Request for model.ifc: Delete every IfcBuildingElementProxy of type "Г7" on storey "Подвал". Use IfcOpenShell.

First a look at what the model holds.

```python
import ifcopenshell
import ifcopenshell.util.element

model = ifcopenshell.open("model.ifc")
print(model.schema)
storey = next(s for s in model.by_type("IfcBuildingStorey") if s.Name == "Подвал")
proxies = [e for e in ifcopenshell.util.element.get_decomposition(storey) if e.is_a("IfcBuildingElementProxy")]
seen = {}
for e in proxies:
    element_type = ifcopenshell.util.element.get_type(e)
    name = element_type.Name if element_type not in (None, e) else None
    seen[name] = seen.get(name, 0) + 1
for name, count in sorted(seen.items(), key=str):
    print(count, "x", name)
```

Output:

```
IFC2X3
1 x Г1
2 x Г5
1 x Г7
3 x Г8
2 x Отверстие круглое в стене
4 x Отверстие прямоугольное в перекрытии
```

```python
import ifcopenshell
import ifcopenshell.api.root
import ifcopenshell.util.element

model = ifcopenshell.open("model.ifc")

storey = next(s for s in model.by_type("IfcBuildingStorey") if s.Name == "Подвал")
proxies = [e for e in ifcopenshell.util.element.get_decomposition(storey) if e.is_a("IfcBuildingElementProxy")]
targets = [e for e in proxies if (t := ifcopenshell.util.element.get_type(e)) not in (None, e) and t.Name == "Г7"]

for e in targets:
    ifcopenshell.api.root.remove_product(model, product=e)
print(len(targets), "removed")

model.write("model-out.ifc")
```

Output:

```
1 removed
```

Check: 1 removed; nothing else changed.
